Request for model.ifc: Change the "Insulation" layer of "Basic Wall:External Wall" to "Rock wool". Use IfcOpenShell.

First a look at what the model holds.

```python
import ifcopenshell
import ifcopenshell.util.element

model = ifcopenshell.open("model.ifc")
print(model.schema)
for layer_set in model.by_type("IfcMaterialLayerSet"):
    if layer_set.LayerSetName == "Basic Wall:External Wall":
        for layer in layer_set.MaterialLayers:
            print(layer.id(), layer.Material and layer.Material.Name, layer.LayerThickness, sep=" | ")
        print(len(ifcopenshell.util.element.get_elements_by_material(model, layer_set)), "elements and types use it")
print(sorted(m.Name for m in model.by_type("IfcMaterial") if m.Name)[:60])
```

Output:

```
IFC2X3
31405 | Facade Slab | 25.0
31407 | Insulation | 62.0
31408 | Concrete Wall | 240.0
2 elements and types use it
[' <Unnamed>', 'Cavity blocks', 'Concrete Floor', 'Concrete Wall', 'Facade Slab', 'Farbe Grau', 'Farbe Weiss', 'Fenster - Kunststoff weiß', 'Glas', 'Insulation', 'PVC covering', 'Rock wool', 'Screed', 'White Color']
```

```python
import ifcopenshell
import ifcopenshell.api.material

model = ifcopenshell.open("model.ifc")

layer_set = next(s for s in model.by_type("IfcMaterialLayerSet") if s.LayerSetName == "Basic Wall:External Wall")
layer = next(l for l in layer_set.MaterialLayers if l.Material and l.Material.Name == "Insulation")
material = next(m for m in model.by_type("IfcMaterial") if m.Name == "Rock wool")

# Point this one layer at the other material; renaming the old one would change it everywhere.
ifcopenshell.api.material.edit_layer(model, layer=layer, attributes={}, material=material)

print([l.Material.Name if l.Material else None for l in layer_set.MaterialLayers])

model.write("model_rev.ifc")
```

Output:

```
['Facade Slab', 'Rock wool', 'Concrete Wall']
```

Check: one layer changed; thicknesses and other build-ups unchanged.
